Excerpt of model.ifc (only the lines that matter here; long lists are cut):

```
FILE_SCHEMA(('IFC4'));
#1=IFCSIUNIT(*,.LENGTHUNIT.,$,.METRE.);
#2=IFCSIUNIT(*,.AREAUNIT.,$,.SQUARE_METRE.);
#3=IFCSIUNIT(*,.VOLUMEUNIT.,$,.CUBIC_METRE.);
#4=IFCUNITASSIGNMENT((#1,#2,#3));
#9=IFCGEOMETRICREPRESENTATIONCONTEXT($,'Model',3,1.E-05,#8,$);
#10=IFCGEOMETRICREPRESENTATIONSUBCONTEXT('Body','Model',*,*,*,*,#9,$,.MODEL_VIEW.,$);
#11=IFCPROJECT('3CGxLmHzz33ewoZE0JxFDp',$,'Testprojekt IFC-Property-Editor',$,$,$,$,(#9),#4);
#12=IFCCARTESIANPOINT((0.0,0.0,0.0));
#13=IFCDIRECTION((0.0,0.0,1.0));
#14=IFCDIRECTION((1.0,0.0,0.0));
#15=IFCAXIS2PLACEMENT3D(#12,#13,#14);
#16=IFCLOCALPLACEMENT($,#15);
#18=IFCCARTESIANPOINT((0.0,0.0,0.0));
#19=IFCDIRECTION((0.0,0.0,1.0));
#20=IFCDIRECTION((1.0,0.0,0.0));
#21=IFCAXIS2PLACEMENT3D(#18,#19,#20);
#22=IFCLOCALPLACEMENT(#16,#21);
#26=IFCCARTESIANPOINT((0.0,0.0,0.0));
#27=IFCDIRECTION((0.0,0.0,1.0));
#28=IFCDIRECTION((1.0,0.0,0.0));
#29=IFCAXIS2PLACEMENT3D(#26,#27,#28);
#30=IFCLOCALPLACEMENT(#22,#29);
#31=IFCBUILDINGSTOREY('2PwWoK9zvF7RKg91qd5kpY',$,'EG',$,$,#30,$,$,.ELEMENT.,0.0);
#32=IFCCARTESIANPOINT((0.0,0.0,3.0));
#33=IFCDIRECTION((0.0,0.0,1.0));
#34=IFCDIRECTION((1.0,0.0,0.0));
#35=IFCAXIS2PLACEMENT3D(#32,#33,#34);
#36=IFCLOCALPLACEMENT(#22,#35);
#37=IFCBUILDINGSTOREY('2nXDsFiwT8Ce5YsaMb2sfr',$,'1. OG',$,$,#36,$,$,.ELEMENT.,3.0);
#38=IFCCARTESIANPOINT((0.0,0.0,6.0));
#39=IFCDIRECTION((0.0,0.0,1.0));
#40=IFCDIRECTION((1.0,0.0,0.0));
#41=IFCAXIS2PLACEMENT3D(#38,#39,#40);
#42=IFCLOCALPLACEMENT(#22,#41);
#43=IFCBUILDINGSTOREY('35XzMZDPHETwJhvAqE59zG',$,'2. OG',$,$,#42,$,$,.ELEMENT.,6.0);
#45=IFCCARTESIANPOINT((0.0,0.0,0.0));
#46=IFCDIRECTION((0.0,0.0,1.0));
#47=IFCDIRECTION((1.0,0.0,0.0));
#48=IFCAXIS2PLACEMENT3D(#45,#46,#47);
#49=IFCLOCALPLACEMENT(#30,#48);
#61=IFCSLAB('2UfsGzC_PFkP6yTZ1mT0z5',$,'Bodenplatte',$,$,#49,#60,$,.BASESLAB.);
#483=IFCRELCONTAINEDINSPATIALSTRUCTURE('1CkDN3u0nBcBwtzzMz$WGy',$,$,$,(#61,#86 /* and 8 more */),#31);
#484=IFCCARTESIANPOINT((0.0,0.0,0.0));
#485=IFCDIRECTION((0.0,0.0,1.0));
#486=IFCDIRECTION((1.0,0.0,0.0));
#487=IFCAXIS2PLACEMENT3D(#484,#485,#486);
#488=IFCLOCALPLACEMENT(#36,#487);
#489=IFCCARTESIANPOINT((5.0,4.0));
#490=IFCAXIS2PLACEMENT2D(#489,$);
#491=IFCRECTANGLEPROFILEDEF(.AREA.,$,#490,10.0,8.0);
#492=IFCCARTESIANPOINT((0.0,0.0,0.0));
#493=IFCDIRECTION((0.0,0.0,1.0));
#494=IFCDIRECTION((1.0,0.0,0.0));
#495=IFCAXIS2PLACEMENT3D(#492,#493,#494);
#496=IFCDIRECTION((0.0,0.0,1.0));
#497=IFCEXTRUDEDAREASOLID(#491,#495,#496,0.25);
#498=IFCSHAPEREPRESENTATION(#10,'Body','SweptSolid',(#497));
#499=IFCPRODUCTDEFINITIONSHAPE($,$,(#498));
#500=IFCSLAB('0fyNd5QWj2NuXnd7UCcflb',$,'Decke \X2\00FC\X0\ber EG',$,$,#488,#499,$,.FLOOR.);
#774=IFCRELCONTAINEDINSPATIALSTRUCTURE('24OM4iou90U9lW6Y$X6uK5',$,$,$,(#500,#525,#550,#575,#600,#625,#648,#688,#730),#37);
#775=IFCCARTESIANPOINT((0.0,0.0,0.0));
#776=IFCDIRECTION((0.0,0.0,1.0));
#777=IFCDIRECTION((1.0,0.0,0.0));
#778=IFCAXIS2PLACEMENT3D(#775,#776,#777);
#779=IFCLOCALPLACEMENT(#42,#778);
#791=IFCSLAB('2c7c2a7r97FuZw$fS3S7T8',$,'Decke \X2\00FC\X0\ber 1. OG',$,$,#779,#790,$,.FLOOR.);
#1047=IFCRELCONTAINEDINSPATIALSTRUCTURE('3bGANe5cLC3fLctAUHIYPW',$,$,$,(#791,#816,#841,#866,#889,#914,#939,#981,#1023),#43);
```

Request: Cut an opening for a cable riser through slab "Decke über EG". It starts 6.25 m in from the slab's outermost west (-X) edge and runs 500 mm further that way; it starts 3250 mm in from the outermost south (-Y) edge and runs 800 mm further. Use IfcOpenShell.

```python
import numpy as np
import ifcopenshell
import ifcopenshell.api.feature
import ifcopenshell.api.geometry
import ifcopenshell.api.root
import ifcopenshell.geom
import ifcopenshell.util.placement
import ifcopenshell.util.representation
import ifcopenshell.util.shape
import ifcopenshell.util.unit

model = ifcopenshell.open("model.ifc")
unit_scale = ifcopenshell.util.unit.calculate_unit_scale(model)
settings = ifcopenshell.geom.settings()


def volume(element):
    """Net volume in cubic metres, openings subtracted."""
    shape = ifcopenshell.geom.create_shape(settings, element)
    return ifcopenshell.util.shape.get_volume(shape.geometry)


slab = model.by_id(500)
before = volume(slab)

# Extent in the slab's own axes, in metres. The edges named are its -X and -Y sides.
slab_shape = ifcopenshell.geom.create_shape(settings, slab)
vertices = ifcopenshell.util.shape.get_vertices(slab_shape.geometry)
x_min, y_min, bottom = vertices.min(axis=0)
top = vertices[:, 2].max()

opening = ifcopenshell.api.root.create_entity(model, ifc_class="IfcOpeningElement", name="Cable riser opening", predefined_type="OPENING")
context = ifcopenshell.util.representation.get_context(model, "Model", "Body", "MODEL_VIEW")
width, depth = 0.5, 0.8
outline = [(0.0, 0.0), (width, 0.0), (width, depth), (0.0, depth), (0.0, 0.0)]
# Overshoot both faces by 50 mm so the cut is clean.
shape = ifcopenshell.api.geometry.add_slab_representation(
    model, context=context, depth=top - bottom + 0.1, polyline=outline
)
ifcopenshell.api.geometry.assign_representation(model, product=opening, representation=shape)

matrix = ifcopenshell.util.placement.get_local_placement(slab.ObjectPlacement)
matrix[:, 3] = matrix @ np.append(np.array([x_min + 6.25, y_min + 3.25, bottom - 0.05]) / unit_scale, 1.0)
ifcopenshell.api.geometry.edit_object_placement(model, product=opening, matrix=matrix, is_si=False)
ifcopenshell.api.feature.add_feature(model, feature=opening, element=slab)

after = volume(slab)

print(f"slab volume {before:.3f} -> {after:.3f} m3")

model.write("model_v2.ifc")
```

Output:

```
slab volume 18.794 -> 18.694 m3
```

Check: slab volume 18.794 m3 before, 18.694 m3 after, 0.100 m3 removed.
